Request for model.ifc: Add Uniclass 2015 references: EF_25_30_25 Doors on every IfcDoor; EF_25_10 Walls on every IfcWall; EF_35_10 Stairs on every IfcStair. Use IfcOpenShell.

First a look at what the model holds.

```python
import ifcopenshell

model = ifcopenshell.open("model.ifc")
print(model.schema)
print("classifications:", [c.Name for c in model.by_type("IfcClassification")])
for ifc_class in ("IfcDoor", "IfcRoof", "IfcStair", "IfcWall", "IfcWindow"):
    print(ifc_class, len(model.by_type(ifc_class)))
```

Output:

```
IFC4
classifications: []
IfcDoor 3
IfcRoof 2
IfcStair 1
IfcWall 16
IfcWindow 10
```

```python
import ifcopenshell
import ifcopenshell.api.classification

model = ifcopenshell.open("model.ifc")

system = ifcopenshell.api.classification.add_classification(model, classification="Uniclass 2015")

codes = {
    "IfcDoor": ("EF_25_30_25", "Doors"),
    "IfcWall": ("EF_25_10", "Walls"),
    "IfcStair": ("EF_35_10", "Stairs"),
}
for ifc_class, (code, name) in codes.items():
    products = model.by_type(ifc_class)
    ifcopenshell.api.classification.add_reference(
        model, products=products, classification=system, identification=code, name=name
    )
    print(code, len(products))

model.write("model_rev.ifc")
```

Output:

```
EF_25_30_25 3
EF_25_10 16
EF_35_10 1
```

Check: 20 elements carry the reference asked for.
